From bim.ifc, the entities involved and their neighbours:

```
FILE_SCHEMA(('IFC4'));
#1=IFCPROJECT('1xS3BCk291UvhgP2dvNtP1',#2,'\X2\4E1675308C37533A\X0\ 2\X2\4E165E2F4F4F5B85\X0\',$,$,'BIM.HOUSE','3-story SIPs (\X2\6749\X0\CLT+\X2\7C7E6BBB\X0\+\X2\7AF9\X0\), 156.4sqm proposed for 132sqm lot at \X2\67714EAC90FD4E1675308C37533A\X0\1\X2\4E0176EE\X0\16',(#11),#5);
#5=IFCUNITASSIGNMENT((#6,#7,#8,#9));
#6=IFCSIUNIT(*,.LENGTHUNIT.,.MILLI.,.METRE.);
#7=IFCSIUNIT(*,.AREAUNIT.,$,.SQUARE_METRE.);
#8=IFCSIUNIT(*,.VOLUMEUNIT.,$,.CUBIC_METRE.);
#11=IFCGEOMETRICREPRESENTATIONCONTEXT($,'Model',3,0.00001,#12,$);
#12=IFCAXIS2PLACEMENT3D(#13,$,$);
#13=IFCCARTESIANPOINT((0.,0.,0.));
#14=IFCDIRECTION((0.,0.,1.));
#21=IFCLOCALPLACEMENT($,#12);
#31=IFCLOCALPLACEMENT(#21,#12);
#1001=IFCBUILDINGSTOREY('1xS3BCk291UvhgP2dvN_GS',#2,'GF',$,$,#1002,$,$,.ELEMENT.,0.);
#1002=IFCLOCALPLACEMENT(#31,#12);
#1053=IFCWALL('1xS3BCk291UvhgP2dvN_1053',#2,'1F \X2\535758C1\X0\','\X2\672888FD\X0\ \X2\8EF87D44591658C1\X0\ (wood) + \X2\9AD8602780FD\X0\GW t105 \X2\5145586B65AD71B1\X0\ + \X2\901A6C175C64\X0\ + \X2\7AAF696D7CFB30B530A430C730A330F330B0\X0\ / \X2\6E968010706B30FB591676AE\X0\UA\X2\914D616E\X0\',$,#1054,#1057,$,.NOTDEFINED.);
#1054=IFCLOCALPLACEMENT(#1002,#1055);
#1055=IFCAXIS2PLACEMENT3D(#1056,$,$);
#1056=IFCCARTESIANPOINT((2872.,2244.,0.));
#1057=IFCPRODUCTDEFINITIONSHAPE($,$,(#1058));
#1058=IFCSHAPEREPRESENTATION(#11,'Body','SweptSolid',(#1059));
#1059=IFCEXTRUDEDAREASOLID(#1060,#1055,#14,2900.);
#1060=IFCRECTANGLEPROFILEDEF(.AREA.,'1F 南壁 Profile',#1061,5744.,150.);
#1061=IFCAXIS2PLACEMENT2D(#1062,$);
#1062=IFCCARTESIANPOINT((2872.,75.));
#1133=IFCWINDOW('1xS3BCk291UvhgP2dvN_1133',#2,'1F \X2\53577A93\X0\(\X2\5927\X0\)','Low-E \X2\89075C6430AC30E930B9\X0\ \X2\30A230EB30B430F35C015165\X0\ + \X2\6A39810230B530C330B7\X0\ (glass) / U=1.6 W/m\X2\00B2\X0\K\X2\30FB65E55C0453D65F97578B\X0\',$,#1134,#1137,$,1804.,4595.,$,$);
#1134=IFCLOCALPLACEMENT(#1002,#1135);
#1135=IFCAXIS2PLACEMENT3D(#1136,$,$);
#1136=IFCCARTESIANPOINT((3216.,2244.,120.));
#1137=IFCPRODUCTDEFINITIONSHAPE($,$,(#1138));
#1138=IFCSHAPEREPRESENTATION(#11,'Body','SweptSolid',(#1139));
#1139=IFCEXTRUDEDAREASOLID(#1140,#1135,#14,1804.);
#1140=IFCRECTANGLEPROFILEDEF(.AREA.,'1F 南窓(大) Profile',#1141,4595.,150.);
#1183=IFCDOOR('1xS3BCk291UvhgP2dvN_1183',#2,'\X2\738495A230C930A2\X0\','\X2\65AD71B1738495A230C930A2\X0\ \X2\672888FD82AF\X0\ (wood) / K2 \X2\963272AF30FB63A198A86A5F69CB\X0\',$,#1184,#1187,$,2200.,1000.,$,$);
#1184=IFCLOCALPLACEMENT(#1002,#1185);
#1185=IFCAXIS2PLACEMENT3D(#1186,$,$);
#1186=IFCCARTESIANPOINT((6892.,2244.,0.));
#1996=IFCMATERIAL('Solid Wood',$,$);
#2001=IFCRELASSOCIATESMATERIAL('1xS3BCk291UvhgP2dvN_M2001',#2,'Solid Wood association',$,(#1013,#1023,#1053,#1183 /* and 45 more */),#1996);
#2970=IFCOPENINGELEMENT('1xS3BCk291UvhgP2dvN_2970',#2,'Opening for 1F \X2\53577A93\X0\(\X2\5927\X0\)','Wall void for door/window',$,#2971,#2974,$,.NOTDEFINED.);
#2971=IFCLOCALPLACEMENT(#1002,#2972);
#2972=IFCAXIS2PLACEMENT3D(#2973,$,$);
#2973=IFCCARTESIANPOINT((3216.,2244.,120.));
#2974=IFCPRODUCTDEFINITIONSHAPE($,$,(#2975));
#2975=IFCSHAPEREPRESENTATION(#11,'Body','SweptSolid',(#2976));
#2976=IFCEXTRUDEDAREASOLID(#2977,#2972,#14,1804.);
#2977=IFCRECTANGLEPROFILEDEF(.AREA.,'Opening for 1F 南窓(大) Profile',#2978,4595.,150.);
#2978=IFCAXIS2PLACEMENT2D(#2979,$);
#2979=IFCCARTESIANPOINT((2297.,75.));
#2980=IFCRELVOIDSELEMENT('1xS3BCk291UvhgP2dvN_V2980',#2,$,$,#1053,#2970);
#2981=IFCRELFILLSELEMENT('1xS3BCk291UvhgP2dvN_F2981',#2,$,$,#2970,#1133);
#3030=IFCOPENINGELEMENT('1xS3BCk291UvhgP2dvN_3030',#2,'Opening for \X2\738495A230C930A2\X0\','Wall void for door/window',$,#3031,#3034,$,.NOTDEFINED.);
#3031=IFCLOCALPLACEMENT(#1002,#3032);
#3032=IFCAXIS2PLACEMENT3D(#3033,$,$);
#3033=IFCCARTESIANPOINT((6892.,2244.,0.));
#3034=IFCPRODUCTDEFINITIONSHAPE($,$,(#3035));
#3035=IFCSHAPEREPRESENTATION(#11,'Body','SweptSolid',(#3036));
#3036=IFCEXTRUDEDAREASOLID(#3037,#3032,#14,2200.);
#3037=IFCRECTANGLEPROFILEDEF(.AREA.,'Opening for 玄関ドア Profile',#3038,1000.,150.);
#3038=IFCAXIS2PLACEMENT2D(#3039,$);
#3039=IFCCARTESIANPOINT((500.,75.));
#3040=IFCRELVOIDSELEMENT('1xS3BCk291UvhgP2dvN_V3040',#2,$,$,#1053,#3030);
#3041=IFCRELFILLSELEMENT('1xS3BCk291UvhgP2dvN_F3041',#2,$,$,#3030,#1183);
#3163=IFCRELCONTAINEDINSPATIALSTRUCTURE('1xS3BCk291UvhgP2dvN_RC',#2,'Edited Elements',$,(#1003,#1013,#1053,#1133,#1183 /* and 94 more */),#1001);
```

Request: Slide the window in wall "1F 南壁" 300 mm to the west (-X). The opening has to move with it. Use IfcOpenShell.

```python
import ifcopenshell
import ifcopenshell.api.geometry
import ifcopenshell.util.placement
import ifcopenshell.util.unit

model = ifcopenshell.open("bim.ifc")
unit_scale = ifcopenshell.util.unit.calculate_unit_scale(model)

window = model.by_guid("1xS3BCk291UvhgP2dvN_1133")
opening = window.FillsVoids[0].RelatingOpeningElement
wall = opening.VoidsElements[0].RelatingBuildingElement

wall_matrix = ifcopenshell.util.placement.get_local_placement(wall.ObjectPlacement)
shift = wall_matrix[:3, 0] * -0.3 / unit_scale
before = ifcopenshell.util.placement.get_local_placement(window.ObjectPlacement)[:3, 3].copy()

# The window is not placed relative to its opening, so move both.
for product in (opening, window):
    matrix = ifcopenshell.util.placement.get_local_placement(product.ObjectPlacement)
    matrix[:3, 3] += shift
    ifcopenshell.api.geometry.edit_object_placement(model, product=product, matrix=matrix, is_si=False)

after = ifcopenshell.util.placement.get_local_placement(window.ObjectPlacement)[:3, 3]
print("window moved by", (after - before).round(3) + 0.0)

model.write("bim_updated.ifc")
```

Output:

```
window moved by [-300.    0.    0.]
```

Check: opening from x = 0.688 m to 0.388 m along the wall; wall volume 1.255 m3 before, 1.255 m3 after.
